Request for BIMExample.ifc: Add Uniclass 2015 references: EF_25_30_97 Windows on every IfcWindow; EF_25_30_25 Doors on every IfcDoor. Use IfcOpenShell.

First a look at what the model holds.

```python
import ifcopenshell

model = ifcopenshell.open("BIMExample.ifc")
print(model.schema)
print("classifications:", [c.Name for c in model.by_type("IfcClassification")])
for ifc_class in ("IfcDoor", "IfcRoof", "IfcStair", "IfcWall", "IfcWindow"):
    print(ifc_class, len(model.by_type(ifc_class)))
```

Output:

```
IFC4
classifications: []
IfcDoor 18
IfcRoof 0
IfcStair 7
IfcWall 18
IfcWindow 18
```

```python
import ifcopenshell
import ifcopenshell.api.classification

model = ifcopenshell.open("BIMExample.ifc")

system = ifcopenshell.api.classification.add_classification(model, classification="Uniclass 2015")

codes = {
    "IfcWindow": ("EF_25_30_97", "Windows"),
    "IfcDoor": ("EF_25_30_25", "Doors"),
}
for ifc_class, (code, name) in codes.items():
    products = model.by_type(ifc_class)
    ifcopenshell.api.classification.add_reference(
        model, products=products, classification=system, identification=code, name=name
    )
    print(code, len(products))

model.write("BIMExample_rev.ifc")
```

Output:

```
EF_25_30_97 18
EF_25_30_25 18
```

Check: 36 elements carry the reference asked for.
